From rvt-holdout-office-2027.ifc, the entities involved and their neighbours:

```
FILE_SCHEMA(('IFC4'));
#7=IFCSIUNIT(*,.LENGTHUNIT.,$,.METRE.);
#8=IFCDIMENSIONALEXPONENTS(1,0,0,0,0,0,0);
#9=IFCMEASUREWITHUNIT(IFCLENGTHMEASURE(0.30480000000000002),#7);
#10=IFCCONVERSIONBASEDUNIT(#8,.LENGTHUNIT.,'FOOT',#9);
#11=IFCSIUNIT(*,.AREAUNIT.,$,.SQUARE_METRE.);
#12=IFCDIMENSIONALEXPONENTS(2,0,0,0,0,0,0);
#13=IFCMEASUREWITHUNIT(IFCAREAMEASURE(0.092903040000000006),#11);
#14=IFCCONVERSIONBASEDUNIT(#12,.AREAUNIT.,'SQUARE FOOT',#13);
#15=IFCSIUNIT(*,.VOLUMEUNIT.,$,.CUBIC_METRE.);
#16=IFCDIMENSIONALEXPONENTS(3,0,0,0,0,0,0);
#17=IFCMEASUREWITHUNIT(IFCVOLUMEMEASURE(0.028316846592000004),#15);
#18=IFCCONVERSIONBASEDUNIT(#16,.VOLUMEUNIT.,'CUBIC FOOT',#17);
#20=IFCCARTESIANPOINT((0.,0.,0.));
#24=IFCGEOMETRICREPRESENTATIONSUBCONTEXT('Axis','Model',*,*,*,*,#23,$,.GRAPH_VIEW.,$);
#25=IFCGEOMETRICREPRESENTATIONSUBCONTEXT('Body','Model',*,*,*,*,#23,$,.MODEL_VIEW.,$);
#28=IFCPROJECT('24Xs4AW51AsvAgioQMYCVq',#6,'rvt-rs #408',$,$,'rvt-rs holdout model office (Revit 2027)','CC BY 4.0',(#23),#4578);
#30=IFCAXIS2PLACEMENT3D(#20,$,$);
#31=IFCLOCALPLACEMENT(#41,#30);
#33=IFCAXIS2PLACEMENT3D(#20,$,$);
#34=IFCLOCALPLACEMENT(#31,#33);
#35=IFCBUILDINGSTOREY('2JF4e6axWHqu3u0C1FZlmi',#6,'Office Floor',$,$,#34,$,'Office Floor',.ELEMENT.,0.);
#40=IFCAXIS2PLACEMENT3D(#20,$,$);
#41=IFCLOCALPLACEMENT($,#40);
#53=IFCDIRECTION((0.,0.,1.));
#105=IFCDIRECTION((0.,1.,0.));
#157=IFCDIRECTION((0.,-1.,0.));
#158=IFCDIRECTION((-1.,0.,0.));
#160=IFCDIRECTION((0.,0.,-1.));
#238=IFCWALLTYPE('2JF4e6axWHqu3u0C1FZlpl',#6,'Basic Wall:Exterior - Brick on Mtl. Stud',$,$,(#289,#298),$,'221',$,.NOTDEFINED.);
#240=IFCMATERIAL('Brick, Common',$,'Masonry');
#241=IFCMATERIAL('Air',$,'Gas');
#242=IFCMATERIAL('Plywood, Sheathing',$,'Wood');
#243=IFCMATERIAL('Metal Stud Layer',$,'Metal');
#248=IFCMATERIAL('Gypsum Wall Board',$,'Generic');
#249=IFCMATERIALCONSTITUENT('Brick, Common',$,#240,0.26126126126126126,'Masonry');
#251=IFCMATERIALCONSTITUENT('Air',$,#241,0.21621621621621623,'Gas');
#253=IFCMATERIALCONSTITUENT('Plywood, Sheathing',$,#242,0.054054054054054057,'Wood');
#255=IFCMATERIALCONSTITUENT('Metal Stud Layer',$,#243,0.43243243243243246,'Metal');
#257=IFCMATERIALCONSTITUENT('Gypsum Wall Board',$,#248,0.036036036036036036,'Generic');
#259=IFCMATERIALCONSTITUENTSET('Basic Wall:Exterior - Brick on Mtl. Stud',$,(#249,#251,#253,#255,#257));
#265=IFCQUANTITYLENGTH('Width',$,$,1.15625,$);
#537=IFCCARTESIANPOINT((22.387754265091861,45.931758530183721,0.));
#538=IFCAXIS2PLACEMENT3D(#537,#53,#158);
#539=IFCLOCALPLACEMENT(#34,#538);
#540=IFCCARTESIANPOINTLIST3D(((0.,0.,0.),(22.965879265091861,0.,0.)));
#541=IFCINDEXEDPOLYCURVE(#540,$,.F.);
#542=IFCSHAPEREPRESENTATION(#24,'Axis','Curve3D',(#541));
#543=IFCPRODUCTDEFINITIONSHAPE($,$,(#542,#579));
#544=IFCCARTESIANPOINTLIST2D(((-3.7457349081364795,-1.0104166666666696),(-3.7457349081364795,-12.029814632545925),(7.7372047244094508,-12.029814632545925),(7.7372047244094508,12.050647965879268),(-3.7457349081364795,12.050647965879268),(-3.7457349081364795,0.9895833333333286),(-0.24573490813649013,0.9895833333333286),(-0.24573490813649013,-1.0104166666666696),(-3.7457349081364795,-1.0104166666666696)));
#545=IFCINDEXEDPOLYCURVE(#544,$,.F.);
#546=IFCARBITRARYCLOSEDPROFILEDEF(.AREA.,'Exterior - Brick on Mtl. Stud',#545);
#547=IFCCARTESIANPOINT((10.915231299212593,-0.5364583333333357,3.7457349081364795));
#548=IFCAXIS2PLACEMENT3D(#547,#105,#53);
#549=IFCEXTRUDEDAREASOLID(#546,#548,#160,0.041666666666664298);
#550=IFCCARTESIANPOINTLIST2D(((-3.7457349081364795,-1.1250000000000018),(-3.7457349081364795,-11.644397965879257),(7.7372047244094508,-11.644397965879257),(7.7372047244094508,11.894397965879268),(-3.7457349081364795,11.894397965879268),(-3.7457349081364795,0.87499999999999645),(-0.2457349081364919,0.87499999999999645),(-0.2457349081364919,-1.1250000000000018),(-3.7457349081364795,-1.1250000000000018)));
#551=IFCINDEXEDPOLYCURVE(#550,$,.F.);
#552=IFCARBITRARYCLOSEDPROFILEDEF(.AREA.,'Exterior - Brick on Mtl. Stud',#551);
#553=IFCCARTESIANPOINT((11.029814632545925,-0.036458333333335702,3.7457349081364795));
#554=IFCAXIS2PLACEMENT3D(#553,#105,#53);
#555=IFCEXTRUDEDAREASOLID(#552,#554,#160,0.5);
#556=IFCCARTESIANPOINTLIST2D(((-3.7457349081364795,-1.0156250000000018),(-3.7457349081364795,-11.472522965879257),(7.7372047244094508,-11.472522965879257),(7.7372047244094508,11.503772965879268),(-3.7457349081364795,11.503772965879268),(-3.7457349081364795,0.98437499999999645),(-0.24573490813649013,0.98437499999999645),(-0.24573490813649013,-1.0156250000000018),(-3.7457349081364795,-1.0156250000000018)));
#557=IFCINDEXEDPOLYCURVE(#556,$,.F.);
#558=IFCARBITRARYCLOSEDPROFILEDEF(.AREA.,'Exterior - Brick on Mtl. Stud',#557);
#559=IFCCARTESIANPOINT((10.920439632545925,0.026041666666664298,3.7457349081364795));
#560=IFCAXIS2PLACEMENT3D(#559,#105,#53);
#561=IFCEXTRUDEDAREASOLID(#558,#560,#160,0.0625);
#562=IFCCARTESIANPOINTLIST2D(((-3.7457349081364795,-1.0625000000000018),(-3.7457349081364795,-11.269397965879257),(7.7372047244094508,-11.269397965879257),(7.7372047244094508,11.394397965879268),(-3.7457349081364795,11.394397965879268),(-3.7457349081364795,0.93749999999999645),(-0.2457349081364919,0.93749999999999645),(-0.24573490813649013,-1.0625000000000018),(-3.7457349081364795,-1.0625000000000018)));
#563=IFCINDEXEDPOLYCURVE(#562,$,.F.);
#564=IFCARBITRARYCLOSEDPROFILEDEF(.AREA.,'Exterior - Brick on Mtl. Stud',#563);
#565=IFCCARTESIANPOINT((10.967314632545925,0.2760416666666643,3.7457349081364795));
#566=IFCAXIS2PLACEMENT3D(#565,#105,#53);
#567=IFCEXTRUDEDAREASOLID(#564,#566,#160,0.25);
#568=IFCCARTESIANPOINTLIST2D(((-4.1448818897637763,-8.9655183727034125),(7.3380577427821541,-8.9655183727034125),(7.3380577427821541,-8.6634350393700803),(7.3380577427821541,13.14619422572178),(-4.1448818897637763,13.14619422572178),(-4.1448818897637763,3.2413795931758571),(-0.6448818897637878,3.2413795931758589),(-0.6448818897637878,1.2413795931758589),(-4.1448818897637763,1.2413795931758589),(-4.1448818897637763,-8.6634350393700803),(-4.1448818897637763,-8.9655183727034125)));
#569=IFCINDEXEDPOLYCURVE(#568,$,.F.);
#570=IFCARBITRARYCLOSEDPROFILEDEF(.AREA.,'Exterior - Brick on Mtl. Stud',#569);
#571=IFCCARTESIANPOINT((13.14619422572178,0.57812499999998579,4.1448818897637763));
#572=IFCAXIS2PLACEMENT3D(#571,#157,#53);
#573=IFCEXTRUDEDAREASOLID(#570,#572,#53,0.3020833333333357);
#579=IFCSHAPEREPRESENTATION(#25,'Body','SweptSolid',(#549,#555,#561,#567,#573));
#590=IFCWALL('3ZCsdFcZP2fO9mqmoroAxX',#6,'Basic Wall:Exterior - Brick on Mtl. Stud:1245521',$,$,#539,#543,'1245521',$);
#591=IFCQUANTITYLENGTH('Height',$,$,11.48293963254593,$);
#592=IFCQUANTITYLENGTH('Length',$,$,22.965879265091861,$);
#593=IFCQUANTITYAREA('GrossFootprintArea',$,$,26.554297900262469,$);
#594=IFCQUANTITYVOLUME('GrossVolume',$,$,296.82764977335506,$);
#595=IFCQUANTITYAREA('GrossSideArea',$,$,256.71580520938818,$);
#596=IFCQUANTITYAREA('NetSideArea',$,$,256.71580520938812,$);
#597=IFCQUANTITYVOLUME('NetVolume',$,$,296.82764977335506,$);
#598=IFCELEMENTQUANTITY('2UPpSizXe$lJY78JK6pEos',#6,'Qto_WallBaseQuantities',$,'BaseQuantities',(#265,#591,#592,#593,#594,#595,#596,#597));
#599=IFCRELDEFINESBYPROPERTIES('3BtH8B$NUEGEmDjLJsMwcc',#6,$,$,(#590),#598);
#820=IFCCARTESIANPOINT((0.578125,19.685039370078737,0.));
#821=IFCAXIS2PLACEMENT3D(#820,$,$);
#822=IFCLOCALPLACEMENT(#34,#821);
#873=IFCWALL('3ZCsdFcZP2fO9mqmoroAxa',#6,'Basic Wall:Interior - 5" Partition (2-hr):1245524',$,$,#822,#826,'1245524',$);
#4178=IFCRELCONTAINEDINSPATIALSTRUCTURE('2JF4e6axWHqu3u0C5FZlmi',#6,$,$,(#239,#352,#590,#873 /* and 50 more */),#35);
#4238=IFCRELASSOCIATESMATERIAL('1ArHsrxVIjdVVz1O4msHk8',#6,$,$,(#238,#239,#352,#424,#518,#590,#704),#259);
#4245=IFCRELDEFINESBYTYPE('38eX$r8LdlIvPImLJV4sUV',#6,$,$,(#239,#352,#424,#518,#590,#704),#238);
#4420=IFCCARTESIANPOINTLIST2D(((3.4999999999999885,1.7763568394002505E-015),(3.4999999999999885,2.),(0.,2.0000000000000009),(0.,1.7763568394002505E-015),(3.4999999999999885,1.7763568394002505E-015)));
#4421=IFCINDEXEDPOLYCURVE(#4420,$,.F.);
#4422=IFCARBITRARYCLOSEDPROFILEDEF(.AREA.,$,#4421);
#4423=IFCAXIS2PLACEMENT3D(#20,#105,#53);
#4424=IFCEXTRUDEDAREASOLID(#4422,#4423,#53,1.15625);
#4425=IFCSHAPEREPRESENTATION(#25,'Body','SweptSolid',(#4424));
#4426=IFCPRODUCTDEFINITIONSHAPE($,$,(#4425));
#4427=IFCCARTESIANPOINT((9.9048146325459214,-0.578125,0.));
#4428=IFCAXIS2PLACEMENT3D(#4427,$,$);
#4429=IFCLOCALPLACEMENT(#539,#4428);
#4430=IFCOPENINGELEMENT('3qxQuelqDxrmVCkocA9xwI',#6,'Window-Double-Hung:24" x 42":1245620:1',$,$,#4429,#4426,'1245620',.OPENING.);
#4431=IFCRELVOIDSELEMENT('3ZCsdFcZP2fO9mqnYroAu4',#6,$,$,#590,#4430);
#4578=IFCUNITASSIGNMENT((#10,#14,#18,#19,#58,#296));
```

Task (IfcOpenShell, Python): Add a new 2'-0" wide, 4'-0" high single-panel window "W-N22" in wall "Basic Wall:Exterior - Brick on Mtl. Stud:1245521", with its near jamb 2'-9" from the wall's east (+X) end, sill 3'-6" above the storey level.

```python
import numpy as np
import ifcopenshell
import ifcopenshell.api.feature
import ifcopenshell.api.geometry
import ifcopenshell.api.pset
import ifcopenshell.api.root
import ifcopenshell.api.spatial
import ifcopenshell.geom
import ifcopenshell.util.element
import ifcopenshell.util.placement
import ifcopenshell.util.representation
import ifcopenshell.util.shape
import ifcopenshell.util.unit

model = ifcopenshell.open("rvt-holdout-office-2027.ifc")
unit_scale = ifcopenshell.util.unit.calculate_unit_scale(model)
area_scale = ifcopenshell.util.unit.calculate_unit_scale(model, "AREAUNIT")
volume_scale = ifcopenshell.util.unit.calculate_unit_scale(model, "VOLUMEUNIT")
settings = ifcopenshell.geom.settings()


def volume(element):
    """Net volume in cubic metres, openings subtracted."""
    shape = ifcopenshell.geom.create_shape(settings, element)
    return ifcopenshell.util.shape.get_volume(shape.geometry)


wall = model.by_guid("3ZCsdFcZP2fO9mqmoroAxX")
storey = ifcopenshell.util.element.get_container(wall, ifc_class="IfcBuildingStorey")
context = ifcopenshell.util.representation.get_context(model, "Model", "Body", "MODEL_VIEW")
before = volume(wall)

width, height, from_end, sill = 0.6096, 1.2192, 0.8382, 1.0668  # metres

# The wall runs along its own X axis, and the end named is its -X end.
wall_shape = ifcopenshell.geom.create_shape(settings, wall)
x, y, z = ifcopenshell.util.shape.get_vertices(wall_shape.geometry).T
start = x.min() + from_end
face, thickness = float(y.min()), float(y.max() - y.min())
wall_matrix = ifcopenshell.util.placement.get_local_placement(wall.ObjectPlacement)
level = ifcopenshell.util.placement.get_local_placement(storey.ObjectPlacement)[2, 3]


def in_wall(x, y):
    """Placement at x, y metres in the wall's axes, at sill height."""
    matrix = wall_matrix.copy()
    matrix[:, 3] = wall_matrix @ np.array([x / unit_scale, y / unit_scale, 0.0, 1.0])
    matrix[2, 3] = level + sill / unit_scale
    return matrix


# Opening: a box that overshoots both wall faces by 50 mm.
opening = ifcopenshell.api.root.create_entity(model, ifc_class="IfcOpeningElement", predefined_type="OPENING")
box = ifcopenshell.api.geometry.add_wall_representation(
    model, context=context, length=width, height=height, thickness=thickness + 0.1
)
ifcopenshell.api.geometry.assign_representation(model, product=opening, representation=box)
ifcopenshell.api.geometry.edit_object_placement(model, product=opening, matrix=in_wall(start, face - 0.05), is_si=False)
ifcopenshell.api.feature.add_feature(model, feature=opening, element=wall)

window = ifcopenshell.api.root.create_entity(model, ifc_class="IfcWindow", name="W-N22", predefined_type="WINDOW")
window.OverallWidth, window.OverallHeight = width / unit_scale, height / unit_scale
window.PartitioningType = "SINGLE_PANEL"
body = ifcopenshell.api.geometry.add_window_representation(
    model,
    context=context,
    overall_width=window.OverallWidth,
    overall_height=window.OverallHeight,
    partition_type="SINGLE_PANEL",
)
ifcopenshell.api.geometry.assign_representation(model, product=window, representation=body)
ifcopenshell.api.spatial.assign_container(model, products=[window], relating_structure=storey)
ifcopenshell.api.feature.add_filling(model, opening=opening, element=window)

# Centre the window in the wall's thickness.
ifcopenshell.api.geometry.edit_object_placement(model, product=window, matrix=in_wall(start, face), is_si=False)
window_shape = ifcopenshell.geom.create_shape(settings, window)
depth = ifcopenshell.util.shape.get_vertices(window_shape.geometry)[:, 1]
offset = face + thickness / 2 - (depth.min() + depth.max()) / 2
ifcopenshell.api.geometry.edit_object_placement(model, product=window, matrix=in_wall(start, offset), is_si=False)

after = volume(wall)

# Update the wall's stored quantities.
qto = model.by_id(ifcopenshell.util.element.get_pset(wall, "Qto_WallBaseQuantities", should_inherit=False)["id"])
ifcopenshell.api.pset.edit_qto(model, qto=qto, properties={
    "NetSideArea": after / thickness / area_scale,
    "NetVolume": after / volume_scale,
})

print(f"wall volume {before:.3f} -> {after:.3f} m3")

model.write("rvt-holdout-office-2027-out.ifc")
```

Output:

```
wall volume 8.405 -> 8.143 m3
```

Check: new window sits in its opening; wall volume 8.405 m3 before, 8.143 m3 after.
